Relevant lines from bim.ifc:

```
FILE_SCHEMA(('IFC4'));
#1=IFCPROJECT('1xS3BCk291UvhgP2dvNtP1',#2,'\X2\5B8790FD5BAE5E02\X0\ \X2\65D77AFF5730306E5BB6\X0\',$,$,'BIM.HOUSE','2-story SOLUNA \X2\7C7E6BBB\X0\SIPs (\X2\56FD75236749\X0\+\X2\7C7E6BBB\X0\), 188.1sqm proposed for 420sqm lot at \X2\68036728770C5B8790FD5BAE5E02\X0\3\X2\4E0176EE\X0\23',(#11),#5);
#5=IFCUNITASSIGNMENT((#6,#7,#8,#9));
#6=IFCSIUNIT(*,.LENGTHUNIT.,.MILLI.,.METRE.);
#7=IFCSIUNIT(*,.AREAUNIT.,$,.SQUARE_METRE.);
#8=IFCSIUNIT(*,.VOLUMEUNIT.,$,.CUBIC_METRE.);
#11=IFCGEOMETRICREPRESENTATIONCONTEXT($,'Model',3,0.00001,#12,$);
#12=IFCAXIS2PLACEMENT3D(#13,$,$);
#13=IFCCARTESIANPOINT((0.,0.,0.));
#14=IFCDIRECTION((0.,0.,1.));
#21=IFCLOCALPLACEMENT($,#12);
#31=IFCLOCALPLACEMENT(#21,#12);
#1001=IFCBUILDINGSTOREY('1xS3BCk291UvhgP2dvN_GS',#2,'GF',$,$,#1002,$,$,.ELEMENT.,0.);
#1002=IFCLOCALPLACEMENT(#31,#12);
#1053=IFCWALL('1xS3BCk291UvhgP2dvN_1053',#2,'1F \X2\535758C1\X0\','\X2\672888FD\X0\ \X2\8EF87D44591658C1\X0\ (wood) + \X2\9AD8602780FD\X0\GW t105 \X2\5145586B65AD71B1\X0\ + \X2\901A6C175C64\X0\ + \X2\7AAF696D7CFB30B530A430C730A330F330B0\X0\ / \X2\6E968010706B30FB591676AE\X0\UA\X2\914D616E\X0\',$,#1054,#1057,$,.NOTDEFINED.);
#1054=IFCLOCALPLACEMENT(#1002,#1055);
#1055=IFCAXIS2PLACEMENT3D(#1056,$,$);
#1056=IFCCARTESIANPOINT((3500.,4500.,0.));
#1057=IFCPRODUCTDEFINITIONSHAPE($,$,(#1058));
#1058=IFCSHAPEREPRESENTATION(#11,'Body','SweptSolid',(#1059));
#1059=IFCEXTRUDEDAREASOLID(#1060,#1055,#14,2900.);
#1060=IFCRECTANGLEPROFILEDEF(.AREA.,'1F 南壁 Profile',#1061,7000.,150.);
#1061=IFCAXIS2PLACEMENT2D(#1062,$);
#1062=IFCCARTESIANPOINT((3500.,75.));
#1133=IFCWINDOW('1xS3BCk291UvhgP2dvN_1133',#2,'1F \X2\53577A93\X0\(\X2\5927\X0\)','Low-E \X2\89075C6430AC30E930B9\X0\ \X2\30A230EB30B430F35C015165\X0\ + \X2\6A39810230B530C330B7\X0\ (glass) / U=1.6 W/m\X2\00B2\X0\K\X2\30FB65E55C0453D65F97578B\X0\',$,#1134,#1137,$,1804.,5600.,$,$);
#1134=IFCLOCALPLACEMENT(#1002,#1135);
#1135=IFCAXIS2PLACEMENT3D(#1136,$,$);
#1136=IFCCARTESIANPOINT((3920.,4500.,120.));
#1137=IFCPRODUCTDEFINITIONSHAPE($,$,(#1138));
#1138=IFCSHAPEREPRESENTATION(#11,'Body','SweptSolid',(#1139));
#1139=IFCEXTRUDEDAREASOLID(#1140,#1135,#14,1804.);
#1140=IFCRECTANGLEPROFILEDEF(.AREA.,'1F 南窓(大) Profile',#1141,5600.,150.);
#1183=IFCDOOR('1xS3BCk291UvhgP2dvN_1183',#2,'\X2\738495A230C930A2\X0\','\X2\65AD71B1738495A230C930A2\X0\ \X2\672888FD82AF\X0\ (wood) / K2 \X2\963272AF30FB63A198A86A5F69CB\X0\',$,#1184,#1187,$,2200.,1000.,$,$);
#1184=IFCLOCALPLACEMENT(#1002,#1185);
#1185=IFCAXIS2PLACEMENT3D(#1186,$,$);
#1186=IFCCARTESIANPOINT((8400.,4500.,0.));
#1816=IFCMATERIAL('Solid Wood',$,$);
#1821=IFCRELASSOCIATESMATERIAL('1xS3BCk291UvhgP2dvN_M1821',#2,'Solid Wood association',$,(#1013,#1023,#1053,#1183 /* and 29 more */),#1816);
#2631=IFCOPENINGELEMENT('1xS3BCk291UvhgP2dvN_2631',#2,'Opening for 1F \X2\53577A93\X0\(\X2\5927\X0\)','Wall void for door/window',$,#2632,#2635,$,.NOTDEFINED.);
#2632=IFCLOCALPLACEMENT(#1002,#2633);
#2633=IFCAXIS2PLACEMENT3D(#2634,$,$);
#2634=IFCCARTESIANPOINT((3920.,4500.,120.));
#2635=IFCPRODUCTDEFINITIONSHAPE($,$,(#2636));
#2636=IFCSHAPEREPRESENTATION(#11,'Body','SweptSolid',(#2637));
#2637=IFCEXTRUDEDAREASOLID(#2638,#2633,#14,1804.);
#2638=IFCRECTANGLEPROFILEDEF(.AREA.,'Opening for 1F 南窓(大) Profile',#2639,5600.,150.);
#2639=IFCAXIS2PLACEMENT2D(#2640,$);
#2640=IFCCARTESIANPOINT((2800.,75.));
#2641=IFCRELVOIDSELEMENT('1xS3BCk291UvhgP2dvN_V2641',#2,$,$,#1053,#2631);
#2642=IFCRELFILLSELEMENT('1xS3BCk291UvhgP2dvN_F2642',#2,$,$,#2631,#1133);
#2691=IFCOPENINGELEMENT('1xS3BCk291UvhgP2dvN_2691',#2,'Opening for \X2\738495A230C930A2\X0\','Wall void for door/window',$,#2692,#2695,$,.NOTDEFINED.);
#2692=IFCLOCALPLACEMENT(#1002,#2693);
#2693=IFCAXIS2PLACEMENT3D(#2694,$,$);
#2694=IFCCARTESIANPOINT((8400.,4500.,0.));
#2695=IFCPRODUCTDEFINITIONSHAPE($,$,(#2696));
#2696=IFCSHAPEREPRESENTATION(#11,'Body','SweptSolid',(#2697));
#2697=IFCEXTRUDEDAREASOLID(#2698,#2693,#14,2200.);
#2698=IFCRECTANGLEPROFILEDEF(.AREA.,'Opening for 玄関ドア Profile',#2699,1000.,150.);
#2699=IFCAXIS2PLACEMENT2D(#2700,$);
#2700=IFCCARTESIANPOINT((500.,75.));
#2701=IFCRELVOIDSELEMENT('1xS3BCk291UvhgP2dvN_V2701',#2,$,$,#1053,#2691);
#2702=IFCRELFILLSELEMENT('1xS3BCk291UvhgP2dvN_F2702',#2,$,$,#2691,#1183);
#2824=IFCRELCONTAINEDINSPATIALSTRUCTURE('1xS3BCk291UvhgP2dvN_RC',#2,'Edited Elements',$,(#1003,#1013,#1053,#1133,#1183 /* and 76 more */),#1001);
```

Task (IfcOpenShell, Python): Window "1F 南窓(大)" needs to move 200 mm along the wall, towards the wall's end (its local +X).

```python
import ifcopenshell
import ifcopenshell.api.geometry
import ifcopenshell.util.placement
import ifcopenshell.util.unit

model = ifcopenshell.open("bim.ifc")
unit_scale = ifcopenshell.util.unit.calculate_unit_scale(model)

window = model.by_guid("1xS3BCk291UvhgP2dvN_1133")
opening = window.FillsVoids[0].RelatingOpeningElement
wall = opening.VoidsElements[0].RelatingBuildingElement

wall_matrix = ifcopenshell.util.placement.get_local_placement(wall.ObjectPlacement)
shift = wall_matrix[:3, 0] * 0.2 / unit_scale
before = ifcopenshell.util.placement.get_local_placement(window.ObjectPlacement)[:3, 3].copy()

# The window is not placed relative to its opening, so move both.
for product in (opening, window):
    matrix = ifcopenshell.util.placement.get_local_placement(product.ObjectPlacement)
    matrix[:3, 3] += shift
    ifcopenshell.api.geometry.edit_object_placement(model, product=product, matrix=matrix, is_si=False)

after = ifcopenshell.util.placement.get_local_placement(window.ObjectPlacement)[:3, 3]
print("window moved by", (after - before).round(3) + 0.0)

model.write("bim_updated.ifc")
```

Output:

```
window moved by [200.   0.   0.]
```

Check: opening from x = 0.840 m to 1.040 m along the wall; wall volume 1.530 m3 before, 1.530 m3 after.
